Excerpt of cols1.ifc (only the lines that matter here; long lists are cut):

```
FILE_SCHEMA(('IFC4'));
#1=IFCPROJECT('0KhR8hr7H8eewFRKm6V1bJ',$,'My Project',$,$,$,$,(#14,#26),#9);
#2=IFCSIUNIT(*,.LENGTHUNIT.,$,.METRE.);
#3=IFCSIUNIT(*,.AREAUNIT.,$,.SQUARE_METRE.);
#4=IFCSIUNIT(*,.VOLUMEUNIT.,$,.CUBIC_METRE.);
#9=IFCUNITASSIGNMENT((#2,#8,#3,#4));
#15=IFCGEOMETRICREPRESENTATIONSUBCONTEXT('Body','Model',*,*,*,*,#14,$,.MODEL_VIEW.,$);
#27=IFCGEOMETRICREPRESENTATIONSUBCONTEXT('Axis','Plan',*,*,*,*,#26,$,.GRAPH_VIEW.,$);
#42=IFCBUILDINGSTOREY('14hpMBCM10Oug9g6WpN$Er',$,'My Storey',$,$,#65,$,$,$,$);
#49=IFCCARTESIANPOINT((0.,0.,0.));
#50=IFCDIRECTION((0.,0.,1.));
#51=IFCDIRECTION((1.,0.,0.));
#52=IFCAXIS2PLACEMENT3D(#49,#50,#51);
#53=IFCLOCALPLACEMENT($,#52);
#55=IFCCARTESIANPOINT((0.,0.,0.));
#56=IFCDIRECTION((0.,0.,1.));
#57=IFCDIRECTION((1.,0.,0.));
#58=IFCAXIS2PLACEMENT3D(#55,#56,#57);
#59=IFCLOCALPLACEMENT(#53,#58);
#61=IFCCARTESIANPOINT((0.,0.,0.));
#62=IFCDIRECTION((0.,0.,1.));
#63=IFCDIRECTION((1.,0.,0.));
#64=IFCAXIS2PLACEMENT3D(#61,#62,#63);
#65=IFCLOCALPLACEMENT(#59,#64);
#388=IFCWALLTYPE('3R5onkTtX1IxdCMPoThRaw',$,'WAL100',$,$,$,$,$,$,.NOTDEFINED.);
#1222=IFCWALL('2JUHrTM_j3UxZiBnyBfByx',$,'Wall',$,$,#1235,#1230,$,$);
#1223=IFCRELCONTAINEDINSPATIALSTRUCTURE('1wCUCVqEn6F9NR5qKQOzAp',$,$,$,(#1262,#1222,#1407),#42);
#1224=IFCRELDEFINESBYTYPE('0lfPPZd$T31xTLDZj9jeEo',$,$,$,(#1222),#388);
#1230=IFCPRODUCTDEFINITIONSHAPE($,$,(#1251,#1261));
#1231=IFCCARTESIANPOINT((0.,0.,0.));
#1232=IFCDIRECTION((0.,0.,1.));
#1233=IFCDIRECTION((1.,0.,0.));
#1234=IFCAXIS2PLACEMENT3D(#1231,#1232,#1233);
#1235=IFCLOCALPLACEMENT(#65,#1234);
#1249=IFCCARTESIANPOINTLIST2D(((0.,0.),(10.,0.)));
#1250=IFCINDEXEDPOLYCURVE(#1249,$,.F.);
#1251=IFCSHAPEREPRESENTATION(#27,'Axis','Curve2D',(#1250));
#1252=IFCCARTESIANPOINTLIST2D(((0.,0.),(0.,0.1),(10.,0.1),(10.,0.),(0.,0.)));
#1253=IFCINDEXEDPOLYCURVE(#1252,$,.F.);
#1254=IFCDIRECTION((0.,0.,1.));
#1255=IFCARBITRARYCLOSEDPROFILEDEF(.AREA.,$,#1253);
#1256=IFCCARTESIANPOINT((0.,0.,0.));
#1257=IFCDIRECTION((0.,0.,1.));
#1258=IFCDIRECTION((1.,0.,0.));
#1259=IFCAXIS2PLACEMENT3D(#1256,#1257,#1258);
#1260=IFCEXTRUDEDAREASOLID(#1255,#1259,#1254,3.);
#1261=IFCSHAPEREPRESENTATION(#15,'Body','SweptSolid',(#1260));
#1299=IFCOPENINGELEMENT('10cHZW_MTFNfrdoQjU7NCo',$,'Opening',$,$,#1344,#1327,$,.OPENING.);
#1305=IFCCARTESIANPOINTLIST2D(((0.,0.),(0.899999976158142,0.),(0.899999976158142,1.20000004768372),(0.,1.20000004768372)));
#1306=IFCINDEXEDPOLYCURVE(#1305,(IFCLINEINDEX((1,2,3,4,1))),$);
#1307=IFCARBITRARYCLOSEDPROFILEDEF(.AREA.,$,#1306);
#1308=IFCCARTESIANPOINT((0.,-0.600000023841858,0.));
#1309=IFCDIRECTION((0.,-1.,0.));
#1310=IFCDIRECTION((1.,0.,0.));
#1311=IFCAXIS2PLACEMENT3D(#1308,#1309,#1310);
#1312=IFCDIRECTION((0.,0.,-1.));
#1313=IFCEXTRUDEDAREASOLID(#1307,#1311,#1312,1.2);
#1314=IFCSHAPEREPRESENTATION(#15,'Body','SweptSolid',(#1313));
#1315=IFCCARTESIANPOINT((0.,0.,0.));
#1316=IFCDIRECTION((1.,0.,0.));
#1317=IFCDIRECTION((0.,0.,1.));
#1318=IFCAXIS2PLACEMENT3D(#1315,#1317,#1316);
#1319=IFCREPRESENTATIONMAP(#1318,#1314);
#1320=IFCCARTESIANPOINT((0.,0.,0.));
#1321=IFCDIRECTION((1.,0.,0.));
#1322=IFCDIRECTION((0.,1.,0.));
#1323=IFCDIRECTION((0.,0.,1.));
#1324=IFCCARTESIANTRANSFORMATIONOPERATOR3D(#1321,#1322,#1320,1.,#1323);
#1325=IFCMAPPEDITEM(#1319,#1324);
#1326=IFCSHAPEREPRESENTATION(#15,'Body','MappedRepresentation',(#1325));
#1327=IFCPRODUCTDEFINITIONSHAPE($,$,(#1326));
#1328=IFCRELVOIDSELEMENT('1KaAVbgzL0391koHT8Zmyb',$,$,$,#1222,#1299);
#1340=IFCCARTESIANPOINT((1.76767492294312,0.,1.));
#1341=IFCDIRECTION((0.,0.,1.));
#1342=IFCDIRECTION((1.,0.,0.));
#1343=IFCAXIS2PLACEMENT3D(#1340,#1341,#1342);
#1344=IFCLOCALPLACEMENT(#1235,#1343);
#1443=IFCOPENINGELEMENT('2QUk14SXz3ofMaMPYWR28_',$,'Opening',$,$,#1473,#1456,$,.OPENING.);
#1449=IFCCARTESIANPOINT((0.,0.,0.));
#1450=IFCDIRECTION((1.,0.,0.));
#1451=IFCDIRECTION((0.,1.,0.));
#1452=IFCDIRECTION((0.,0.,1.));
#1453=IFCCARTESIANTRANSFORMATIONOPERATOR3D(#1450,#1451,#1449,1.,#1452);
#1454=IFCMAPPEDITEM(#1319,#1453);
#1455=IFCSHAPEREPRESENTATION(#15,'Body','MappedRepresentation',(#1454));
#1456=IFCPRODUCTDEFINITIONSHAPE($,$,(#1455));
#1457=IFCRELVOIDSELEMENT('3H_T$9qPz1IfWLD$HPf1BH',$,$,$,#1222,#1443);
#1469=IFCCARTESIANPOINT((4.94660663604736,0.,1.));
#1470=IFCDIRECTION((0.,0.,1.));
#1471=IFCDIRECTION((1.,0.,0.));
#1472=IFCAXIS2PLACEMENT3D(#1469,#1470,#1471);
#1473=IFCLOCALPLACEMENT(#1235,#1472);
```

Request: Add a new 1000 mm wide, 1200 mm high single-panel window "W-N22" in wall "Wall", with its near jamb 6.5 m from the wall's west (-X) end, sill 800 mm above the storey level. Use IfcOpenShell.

```python
import numpy as np
import ifcopenshell
import ifcopenshell.api.feature
import ifcopenshell.api.geometry
import ifcopenshell.api.root
import ifcopenshell.api.spatial
import ifcopenshell.geom
import ifcopenshell.util.element
import ifcopenshell.util.placement
import ifcopenshell.util.representation
import ifcopenshell.util.shape
import ifcopenshell.util.unit

model = ifcopenshell.open("cols1.ifc")
unit_scale = ifcopenshell.util.unit.calculate_unit_scale(model)
settings = ifcopenshell.geom.settings()


def volume(element):
    """Net volume in cubic metres, openings subtracted."""
    shape = ifcopenshell.geom.create_shape(settings, element)
    return ifcopenshell.util.shape.get_volume(shape.geometry)


wall = model.by_guid("2JUHrTM_j3UxZiBnyBfByx")
storey = ifcopenshell.util.element.get_container(wall, ifc_class="IfcBuildingStorey")
context = ifcopenshell.util.representation.get_context(model, "Model", "Body", "MODEL_VIEW")
before = volume(wall)

width, height, from_end, sill = 1, 1.2, 6.5, 0.8  # metres

# The wall runs along its own X axis, and the end named is its -X end.
wall_shape = ifcopenshell.geom.create_shape(settings, wall)
x, y, z = ifcopenshell.util.shape.get_vertices(wall_shape.geometry).T
start = x.min() + from_end
face, thickness = float(y.min()), float(y.max() - y.min())
wall_matrix = ifcopenshell.util.placement.get_local_placement(wall.ObjectPlacement)
level = ifcopenshell.util.placement.get_local_placement(storey.ObjectPlacement)[2, 3]


def in_wall(x, y):
    """Placement at x, y metres in the wall's axes, at sill height."""
    matrix = wall_matrix.copy()
    matrix[:, 3] = wall_matrix @ np.array([x / unit_scale, y / unit_scale, 0.0, 1.0])
    matrix[2, 3] = level + sill / unit_scale
    return matrix


# Opening: a box that overshoots both wall faces by 50 mm.
opening = ifcopenshell.api.root.create_entity(model, ifc_class="IfcOpeningElement", predefined_type="OPENING")
box = ifcopenshell.api.geometry.add_wall_representation(
    model, context=context, length=width, height=height, thickness=thickness + 0.1
)
ifcopenshell.api.geometry.assign_representation(model, product=opening, representation=box)
ifcopenshell.api.geometry.edit_object_placement(model, product=opening, matrix=in_wall(start, face - 0.05), is_si=False)
ifcopenshell.api.feature.add_feature(model, feature=opening, element=wall)

window = ifcopenshell.api.root.create_entity(model, ifc_class="IfcWindow", name="W-N22", predefined_type="WINDOW")
window.OverallWidth, window.OverallHeight = width / unit_scale, height / unit_scale
window.PartitioningType = "SINGLE_PANEL"
body = ifcopenshell.api.geometry.add_window_representation(
    model,
    context=context,
    overall_width=window.OverallWidth,
    overall_height=window.OverallHeight,
    partition_type="SINGLE_PANEL",
)
ifcopenshell.api.geometry.assign_representation(model, product=window, representation=body)
ifcopenshell.api.spatial.assign_container(model, products=[window], relating_structure=storey)
ifcopenshell.api.feature.add_filling(model, opening=opening, element=window)

# Centre the window in the wall's thickness.
ifcopenshell.api.geometry.edit_object_placement(model, product=window, matrix=in_wall(start, face), is_si=False)
window_shape = ifcopenshell.geom.create_shape(settings, window)
depth = ifcopenshell.util.shape.get_vertices(window_shape.geometry)[:, 1]
offset = face + thickness / 2 - (depth.min() + depth.max()) / 2
ifcopenshell.api.geometry.edit_object_placement(model, product=window, matrix=in_wall(start, offset), is_si=False)

after = volume(wall)

print(f"wall volume {before:.3f} -> {after:.3f} m3")

model.write("cols1-out.ifc")
```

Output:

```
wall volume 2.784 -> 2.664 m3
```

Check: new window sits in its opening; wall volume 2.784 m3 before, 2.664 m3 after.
